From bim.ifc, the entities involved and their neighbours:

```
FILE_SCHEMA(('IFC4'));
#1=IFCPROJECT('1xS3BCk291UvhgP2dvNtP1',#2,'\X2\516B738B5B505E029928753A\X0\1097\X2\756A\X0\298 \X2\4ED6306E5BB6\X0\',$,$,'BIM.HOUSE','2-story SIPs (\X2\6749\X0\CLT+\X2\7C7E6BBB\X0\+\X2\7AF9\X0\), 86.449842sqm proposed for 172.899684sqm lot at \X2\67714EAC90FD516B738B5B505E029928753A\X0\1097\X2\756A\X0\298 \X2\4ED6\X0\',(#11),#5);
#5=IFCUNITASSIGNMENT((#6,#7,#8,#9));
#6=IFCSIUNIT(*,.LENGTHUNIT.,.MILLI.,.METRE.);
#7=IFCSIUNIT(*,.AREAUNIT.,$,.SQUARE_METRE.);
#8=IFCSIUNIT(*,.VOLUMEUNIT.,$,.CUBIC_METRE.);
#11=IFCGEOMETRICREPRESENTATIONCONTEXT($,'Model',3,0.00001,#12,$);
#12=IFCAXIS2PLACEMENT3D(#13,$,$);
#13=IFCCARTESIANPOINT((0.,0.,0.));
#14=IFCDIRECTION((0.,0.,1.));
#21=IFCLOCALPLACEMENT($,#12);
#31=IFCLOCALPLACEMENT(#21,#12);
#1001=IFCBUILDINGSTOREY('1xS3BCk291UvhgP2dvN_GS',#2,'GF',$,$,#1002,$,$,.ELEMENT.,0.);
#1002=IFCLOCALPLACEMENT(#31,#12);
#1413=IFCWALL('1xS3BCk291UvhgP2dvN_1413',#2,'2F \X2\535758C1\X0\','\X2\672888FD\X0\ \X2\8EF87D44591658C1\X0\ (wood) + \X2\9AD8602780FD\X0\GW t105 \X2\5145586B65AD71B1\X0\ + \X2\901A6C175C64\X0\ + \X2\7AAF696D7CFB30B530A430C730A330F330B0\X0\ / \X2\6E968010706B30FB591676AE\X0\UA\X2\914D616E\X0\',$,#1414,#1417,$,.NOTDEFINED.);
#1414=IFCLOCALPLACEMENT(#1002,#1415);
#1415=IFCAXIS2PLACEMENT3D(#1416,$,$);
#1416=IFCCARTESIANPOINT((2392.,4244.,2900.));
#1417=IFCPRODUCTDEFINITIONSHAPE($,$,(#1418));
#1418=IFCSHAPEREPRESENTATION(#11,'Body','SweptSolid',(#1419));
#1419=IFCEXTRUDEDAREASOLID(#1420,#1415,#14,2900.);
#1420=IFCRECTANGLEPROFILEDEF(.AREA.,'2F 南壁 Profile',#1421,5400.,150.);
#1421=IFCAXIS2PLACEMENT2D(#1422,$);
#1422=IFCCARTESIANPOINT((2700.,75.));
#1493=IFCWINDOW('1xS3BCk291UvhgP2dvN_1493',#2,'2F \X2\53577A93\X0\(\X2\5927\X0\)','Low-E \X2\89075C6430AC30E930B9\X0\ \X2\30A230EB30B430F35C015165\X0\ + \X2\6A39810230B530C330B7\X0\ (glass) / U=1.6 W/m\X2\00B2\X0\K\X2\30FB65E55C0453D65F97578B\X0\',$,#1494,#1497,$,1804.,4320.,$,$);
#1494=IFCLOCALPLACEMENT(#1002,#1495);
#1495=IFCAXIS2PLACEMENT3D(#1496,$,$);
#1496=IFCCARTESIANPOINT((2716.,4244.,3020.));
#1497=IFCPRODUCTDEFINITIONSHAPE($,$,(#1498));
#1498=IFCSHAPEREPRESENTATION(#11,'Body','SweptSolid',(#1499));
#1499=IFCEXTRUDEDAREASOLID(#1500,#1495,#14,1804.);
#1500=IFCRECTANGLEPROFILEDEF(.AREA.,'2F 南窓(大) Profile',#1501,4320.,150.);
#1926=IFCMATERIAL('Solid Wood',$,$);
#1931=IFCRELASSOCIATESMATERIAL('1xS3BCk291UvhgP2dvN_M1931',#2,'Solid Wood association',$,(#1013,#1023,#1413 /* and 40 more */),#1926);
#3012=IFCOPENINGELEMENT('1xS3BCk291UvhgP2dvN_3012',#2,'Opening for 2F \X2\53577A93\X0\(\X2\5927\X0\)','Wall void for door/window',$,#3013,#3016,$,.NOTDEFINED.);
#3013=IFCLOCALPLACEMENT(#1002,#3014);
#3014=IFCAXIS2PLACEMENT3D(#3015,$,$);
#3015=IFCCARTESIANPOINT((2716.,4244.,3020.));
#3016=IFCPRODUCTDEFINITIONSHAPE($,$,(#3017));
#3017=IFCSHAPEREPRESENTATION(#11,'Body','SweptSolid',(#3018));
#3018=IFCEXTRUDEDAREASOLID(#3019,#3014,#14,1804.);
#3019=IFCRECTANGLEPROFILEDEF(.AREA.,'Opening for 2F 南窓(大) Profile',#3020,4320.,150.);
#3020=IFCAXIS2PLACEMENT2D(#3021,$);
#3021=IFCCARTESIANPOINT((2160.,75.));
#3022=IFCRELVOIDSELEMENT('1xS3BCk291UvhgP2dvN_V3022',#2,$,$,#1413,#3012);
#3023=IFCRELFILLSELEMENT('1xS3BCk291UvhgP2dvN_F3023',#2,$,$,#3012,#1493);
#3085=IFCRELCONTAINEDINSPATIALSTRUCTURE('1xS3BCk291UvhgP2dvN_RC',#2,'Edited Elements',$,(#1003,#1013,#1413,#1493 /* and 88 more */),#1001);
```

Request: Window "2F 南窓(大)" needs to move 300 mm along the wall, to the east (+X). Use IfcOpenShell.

```python
import ifcopenshell
import ifcopenshell.api.geometry
import ifcopenshell.util.placement
import ifcopenshell.util.unit

model = ifcopenshell.open("bim.ifc")
unit_scale = ifcopenshell.util.unit.calculate_unit_scale(model)

window = model.by_guid("1xS3BCk291UvhgP2dvN_1493")
opening = window.FillsVoids[0].RelatingOpeningElement
wall = opening.VoidsElements[0].RelatingBuildingElement

wall_matrix = ifcopenshell.util.placement.get_local_placement(wall.ObjectPlacement)
shift = wall_matrix[:3, 0] * 0.3 / unit_scale
before = ifcopenshell.util.placement.get_local_placement(window.ObjectPlacement)[:3, 3].copy()

# The window is not placed relative to its opening, so move both.
for product in (opening, window):
    matrix = ifcopenshell.util.placement.get_local_placement(product.ObjectPlacement)
    matrix[:3, 3] += shift
    ifcopenshell.api.geometry.edit_object_placement(model, product=product, matrix=matrix, is_si=False)

after = ifcopenshell.util.placement.get_local_placement(window.ObjectPlacement)[:3, 3]
print("window moved by", (after - before).round(3) + 0.0)

model.write("bim_v2.ifc")
```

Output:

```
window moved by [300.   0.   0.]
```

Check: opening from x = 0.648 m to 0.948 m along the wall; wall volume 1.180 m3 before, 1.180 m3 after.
